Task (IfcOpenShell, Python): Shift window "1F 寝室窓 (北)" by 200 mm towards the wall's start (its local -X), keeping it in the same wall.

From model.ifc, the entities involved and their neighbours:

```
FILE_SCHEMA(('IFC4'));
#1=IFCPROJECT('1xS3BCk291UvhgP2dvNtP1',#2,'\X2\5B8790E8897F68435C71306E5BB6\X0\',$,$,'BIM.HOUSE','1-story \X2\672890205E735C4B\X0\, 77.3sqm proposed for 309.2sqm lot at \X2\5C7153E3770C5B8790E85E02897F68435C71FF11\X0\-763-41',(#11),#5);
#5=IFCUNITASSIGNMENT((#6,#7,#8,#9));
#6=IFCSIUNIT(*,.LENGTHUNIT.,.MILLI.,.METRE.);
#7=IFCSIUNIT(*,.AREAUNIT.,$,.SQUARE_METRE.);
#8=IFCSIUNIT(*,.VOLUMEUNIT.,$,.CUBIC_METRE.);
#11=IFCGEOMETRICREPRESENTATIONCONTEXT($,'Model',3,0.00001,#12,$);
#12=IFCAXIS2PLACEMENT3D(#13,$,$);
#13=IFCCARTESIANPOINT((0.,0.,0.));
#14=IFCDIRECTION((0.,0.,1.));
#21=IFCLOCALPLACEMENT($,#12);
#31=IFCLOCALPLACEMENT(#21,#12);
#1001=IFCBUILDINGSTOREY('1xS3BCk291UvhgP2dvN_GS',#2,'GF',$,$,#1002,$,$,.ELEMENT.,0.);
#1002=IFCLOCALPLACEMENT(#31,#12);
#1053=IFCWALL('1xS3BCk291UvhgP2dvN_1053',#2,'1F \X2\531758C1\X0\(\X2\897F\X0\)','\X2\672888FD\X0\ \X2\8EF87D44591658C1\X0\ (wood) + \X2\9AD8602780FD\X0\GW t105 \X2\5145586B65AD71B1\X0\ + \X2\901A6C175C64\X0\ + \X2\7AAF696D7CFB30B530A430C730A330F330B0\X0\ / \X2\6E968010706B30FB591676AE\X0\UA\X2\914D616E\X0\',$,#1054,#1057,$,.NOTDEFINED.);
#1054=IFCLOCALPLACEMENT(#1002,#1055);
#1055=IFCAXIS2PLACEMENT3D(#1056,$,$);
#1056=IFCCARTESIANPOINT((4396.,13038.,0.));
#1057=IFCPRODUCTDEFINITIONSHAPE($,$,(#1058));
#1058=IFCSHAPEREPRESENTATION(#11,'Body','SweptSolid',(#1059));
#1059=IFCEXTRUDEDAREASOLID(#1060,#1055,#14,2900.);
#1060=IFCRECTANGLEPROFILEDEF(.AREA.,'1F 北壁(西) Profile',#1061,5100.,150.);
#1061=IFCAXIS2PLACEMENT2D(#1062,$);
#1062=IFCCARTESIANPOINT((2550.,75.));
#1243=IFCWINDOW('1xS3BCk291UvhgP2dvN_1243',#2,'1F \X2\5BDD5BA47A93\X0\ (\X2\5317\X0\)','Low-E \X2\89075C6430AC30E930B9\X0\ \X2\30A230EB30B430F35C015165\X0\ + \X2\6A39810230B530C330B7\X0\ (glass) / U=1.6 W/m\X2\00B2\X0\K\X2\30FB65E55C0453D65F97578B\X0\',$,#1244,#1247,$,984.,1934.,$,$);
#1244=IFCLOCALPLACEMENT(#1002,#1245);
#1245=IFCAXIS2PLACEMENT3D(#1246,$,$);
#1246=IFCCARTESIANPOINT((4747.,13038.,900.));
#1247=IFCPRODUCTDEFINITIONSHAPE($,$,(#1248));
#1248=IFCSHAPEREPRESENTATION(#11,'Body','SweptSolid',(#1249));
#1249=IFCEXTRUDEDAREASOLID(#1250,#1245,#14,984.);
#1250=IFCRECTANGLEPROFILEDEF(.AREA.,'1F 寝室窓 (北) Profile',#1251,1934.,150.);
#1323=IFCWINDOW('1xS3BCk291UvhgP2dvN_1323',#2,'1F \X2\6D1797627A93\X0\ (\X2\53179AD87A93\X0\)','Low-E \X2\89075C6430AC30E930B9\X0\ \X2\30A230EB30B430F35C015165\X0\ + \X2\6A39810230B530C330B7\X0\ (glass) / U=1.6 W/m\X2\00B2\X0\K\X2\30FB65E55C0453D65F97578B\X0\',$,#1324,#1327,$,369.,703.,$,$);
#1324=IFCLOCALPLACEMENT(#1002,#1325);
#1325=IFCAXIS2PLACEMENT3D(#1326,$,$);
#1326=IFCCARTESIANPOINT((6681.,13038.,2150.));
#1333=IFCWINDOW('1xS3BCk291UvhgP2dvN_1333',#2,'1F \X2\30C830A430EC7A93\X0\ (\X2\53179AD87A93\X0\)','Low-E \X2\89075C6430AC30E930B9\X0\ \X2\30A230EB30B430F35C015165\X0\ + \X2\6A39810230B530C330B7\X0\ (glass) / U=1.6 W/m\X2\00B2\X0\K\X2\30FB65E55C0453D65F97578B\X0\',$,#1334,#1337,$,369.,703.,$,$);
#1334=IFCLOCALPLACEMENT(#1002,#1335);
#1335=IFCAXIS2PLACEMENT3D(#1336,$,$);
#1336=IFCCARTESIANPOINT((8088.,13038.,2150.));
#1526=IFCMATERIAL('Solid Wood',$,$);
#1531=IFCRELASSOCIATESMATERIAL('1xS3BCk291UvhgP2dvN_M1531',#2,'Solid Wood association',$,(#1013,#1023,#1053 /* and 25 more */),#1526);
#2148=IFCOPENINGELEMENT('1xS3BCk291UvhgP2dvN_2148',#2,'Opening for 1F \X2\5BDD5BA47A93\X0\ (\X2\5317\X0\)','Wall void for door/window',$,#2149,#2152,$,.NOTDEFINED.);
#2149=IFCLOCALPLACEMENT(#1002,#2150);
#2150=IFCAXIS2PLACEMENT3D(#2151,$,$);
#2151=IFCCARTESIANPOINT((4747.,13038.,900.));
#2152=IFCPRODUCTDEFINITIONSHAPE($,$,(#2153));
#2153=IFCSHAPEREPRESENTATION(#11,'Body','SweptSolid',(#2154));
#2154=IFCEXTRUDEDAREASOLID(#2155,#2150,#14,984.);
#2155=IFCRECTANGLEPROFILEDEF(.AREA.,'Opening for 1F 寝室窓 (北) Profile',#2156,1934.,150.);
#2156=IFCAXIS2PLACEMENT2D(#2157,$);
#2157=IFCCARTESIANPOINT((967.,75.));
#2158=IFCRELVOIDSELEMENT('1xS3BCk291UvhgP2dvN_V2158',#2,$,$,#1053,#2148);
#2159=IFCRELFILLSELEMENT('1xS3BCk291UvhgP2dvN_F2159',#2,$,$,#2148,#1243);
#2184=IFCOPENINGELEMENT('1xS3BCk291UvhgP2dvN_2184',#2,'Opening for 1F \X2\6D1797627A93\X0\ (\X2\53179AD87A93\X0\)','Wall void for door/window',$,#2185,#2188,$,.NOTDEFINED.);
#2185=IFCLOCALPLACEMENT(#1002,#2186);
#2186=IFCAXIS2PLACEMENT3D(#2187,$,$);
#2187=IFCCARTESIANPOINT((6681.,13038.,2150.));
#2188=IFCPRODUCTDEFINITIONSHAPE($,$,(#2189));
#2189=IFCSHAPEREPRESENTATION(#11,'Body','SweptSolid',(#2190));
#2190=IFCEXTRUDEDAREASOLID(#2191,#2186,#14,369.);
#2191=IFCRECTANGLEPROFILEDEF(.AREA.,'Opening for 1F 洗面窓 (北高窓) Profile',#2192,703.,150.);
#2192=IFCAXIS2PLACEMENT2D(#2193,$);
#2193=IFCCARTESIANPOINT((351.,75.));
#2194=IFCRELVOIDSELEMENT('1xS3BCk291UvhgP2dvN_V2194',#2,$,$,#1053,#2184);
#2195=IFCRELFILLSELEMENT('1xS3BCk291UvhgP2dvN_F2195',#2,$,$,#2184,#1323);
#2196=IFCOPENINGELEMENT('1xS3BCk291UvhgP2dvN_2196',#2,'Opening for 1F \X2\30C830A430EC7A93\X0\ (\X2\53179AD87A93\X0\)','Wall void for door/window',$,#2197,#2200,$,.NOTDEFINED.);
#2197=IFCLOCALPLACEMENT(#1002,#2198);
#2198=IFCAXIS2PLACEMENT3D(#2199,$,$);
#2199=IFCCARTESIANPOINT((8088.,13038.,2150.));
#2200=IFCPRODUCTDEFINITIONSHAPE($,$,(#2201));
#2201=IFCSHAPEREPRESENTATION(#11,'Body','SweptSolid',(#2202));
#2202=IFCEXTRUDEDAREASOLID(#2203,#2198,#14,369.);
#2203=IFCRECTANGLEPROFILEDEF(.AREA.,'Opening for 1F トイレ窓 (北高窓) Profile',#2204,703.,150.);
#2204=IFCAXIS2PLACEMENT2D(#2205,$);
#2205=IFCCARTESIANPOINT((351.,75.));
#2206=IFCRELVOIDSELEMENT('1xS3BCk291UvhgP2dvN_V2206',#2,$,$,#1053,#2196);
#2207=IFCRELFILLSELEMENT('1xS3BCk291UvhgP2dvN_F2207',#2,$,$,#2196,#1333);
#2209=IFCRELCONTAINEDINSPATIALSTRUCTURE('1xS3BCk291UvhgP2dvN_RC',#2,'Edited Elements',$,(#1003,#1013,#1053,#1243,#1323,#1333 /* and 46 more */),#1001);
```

```python
import ifcopenshell
import ifcopenshell.api.geometry
import ifcopenshell.util.placement

model = ifcopenshell.open("model.ifc")

window = model.by_guid("1xS3BCk291UvhgP2dvN_1243")
opening = window.FillsVoids[0].RelatingOpeningElement
wall = opening.VoidsElements[0].RelatingBuildingElement

wall_matrix = ifcopenshell.util.placement.get_local_placement(wall.ObjectPlacement)
shift = wall_matrix[:3, 0] * -200.0
before = ifcopenshell.util.placement.get_local_placement(window.ObjectPlacement)[:3, 3].copy()

# The window is not placed relative to its opening, so move both.
for product in (opening, window):
    matrix = ifcopenshell.util.placement.get_local_placement(product.ObjectPlacement)
    matrix[:3, 3] += shift
    ifcopenshell.api.geometry.edit_object_placement(model, product=product, matrix=matrix, is_si=False)

after = ifcopenshell.util.placement.get_local_placement(window.ObjectPlacement)[:3, 3]
print("window moved by", (after - before).round(3) + 0.0)

model.write("model_updated.ifc")
```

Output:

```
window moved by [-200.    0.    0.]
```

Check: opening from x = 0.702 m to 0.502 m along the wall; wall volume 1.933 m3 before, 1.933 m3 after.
